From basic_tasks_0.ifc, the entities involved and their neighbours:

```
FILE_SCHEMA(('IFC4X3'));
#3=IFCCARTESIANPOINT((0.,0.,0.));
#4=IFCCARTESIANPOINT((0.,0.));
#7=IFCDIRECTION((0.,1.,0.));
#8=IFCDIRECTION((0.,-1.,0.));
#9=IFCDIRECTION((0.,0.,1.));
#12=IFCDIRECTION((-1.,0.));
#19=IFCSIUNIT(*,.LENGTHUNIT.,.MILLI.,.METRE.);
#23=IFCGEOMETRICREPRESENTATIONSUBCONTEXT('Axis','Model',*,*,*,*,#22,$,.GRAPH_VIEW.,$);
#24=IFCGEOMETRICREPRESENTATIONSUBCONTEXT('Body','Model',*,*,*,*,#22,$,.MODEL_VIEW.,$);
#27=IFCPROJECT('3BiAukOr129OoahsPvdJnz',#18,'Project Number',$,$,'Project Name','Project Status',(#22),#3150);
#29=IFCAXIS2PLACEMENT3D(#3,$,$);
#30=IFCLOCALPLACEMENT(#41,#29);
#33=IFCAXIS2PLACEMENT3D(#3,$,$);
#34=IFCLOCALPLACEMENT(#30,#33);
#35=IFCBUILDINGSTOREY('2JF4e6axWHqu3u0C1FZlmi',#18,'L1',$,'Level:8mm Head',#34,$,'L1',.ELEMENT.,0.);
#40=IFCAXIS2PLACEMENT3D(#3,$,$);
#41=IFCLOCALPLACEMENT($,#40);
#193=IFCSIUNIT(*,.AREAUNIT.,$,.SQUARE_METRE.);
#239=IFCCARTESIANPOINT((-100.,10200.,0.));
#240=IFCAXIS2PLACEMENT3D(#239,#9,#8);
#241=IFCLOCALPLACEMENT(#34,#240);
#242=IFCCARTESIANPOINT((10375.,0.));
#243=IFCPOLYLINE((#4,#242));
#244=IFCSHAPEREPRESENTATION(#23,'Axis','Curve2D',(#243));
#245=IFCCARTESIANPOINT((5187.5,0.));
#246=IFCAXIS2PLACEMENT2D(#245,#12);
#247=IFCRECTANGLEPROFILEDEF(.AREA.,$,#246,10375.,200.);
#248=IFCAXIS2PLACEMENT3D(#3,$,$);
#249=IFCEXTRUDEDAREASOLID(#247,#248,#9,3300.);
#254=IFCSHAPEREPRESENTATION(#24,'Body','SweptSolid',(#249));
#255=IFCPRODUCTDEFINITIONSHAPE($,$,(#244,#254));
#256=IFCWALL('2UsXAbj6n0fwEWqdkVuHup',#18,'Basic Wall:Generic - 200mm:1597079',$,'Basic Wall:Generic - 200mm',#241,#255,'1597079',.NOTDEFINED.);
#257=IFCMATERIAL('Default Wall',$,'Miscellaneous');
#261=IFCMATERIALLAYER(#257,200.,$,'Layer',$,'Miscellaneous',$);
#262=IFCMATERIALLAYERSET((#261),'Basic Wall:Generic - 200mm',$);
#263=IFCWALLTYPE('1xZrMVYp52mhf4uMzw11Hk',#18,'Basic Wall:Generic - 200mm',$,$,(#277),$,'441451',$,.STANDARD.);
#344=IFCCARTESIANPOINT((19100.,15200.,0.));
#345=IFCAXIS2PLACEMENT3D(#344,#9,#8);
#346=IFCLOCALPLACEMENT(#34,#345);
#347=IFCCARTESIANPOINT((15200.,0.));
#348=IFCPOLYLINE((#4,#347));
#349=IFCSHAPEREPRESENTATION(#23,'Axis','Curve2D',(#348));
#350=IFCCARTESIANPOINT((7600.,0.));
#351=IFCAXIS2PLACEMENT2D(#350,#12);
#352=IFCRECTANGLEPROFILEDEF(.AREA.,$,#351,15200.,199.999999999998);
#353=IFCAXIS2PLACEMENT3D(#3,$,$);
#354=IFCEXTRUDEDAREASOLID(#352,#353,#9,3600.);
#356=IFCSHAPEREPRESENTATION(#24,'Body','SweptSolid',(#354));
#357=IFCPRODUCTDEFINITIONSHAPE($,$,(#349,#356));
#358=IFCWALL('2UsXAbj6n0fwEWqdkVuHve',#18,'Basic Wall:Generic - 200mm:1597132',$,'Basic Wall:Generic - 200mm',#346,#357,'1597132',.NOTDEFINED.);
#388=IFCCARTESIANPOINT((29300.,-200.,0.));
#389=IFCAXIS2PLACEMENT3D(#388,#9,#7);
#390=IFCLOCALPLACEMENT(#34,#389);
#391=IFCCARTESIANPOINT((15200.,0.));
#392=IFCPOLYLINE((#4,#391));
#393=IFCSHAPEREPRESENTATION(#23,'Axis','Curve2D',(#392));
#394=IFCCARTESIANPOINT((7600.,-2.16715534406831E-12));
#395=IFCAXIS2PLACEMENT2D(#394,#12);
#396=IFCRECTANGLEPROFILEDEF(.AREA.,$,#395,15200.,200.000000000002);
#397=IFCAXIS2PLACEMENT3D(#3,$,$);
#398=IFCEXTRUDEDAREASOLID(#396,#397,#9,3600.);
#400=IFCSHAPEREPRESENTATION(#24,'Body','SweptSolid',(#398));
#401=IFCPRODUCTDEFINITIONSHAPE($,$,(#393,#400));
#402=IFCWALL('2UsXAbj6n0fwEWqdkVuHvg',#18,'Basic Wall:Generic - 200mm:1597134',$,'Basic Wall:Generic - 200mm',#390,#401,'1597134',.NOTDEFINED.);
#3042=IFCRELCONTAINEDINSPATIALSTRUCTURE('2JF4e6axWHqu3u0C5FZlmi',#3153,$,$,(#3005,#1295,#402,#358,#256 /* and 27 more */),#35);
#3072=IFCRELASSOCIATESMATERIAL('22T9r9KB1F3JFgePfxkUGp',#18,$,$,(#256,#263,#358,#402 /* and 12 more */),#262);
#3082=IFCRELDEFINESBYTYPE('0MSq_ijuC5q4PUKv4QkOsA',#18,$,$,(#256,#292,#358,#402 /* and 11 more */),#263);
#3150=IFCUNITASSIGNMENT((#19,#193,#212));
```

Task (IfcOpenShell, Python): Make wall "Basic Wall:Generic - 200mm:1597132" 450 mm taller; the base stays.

```python
import ifcopenshell
import ifcopenshell.geom
import ifcopenshell.util.representation
import ifcopenshell.util.shape
import ifcopenshell.util.unit

model = ifcopenshell.open("basic_tasks_0.ifc")
unit_scale = ifcopenshell.util.unit.calculate_unit_scale(model)
settings = ifcopenshell.geom.settings()


def volume(element):
    """Net volume in cubic metres, openings subtracted."""
    shape = ifcopenshell.geom.create_shape(settings, element)
    return ifcopenshell.util.shape.get_volume(shape.geometry)


wall = model.by_guid("2UsXAbj6n0fwEWqdkVuHve")
before = volume(wall)

body = ifcopenshell.util.representation.get_representation(wall, "Model", "Body")
solid = body.Items[0]
old_height = solid.Depth
solid.Depth += 0.45 / unit_scale
after = volume(wall)

print(f"height {old_height:g} -> {solid.Depth:g}, volume {before:.3f} -> {after:.3f} m3")

model.write("basic_tasks_0_updated.ifc")
```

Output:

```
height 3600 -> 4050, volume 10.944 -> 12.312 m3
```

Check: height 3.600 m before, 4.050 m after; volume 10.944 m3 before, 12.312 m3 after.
